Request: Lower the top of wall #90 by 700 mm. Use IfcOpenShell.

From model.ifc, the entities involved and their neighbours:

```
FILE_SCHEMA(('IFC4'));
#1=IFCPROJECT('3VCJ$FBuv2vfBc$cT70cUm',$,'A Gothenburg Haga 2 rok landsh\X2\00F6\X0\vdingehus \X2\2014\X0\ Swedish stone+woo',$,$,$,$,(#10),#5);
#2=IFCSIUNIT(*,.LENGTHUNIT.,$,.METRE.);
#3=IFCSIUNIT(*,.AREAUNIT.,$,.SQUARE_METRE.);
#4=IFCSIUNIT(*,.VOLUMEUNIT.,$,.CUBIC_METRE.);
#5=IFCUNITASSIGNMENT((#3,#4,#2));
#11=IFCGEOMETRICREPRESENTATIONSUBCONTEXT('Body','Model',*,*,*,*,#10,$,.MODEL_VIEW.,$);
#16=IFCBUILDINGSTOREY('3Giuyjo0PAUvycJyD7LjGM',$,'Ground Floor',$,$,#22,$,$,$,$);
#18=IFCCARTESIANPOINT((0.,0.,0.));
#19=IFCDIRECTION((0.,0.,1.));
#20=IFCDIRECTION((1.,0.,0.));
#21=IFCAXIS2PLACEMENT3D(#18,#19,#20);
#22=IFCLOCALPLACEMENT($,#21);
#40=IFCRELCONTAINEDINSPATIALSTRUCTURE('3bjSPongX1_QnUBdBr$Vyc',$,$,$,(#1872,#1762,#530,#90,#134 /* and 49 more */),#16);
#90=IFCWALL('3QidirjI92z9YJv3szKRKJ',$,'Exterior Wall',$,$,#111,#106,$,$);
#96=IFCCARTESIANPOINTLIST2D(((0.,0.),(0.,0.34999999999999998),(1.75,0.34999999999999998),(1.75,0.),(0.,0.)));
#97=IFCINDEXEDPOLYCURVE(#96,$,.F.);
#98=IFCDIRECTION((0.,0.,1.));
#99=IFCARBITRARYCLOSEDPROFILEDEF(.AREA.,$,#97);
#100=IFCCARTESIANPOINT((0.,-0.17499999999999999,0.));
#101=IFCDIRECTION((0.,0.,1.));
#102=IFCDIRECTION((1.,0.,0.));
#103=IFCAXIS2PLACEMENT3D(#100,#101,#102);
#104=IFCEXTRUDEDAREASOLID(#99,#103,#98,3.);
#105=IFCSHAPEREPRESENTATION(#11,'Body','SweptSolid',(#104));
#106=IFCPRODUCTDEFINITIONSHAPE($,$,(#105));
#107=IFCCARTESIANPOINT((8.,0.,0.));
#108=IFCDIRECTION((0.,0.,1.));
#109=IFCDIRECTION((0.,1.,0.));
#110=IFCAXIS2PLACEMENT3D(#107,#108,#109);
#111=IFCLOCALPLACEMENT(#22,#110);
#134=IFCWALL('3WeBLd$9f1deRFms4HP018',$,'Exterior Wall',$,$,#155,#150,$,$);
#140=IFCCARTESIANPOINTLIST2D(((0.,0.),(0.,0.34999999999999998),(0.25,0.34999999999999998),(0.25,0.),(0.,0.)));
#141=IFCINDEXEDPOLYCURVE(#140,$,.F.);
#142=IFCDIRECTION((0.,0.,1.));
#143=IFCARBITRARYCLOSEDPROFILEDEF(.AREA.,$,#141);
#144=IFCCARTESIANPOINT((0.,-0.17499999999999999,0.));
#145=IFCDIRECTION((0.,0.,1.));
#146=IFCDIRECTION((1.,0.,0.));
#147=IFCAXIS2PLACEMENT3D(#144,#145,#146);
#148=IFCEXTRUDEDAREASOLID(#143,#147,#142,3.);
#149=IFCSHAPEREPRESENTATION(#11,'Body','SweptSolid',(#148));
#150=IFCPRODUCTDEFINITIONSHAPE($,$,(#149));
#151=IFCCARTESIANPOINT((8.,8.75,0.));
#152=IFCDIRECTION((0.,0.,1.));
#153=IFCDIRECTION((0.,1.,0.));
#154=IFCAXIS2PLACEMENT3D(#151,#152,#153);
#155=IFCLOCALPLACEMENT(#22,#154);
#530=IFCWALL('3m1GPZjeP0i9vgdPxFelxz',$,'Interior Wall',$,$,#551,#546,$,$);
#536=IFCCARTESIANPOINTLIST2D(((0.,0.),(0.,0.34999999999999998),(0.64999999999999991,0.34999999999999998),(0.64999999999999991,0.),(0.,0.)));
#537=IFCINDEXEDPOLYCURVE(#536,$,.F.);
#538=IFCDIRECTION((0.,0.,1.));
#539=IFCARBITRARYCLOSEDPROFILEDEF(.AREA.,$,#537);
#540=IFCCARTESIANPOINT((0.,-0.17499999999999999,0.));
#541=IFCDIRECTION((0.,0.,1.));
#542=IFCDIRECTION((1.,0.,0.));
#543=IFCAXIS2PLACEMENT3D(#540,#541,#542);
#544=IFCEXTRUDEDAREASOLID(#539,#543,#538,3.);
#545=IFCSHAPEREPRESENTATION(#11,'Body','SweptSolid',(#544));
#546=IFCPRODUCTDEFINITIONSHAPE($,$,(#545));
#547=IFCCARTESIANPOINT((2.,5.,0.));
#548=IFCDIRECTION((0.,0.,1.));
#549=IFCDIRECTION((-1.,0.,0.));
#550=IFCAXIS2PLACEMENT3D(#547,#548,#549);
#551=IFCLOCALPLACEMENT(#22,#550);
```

```python
import ifcopenshell
import ifcopenshell.geom
import ifcopenshell.util.representation
import ifcopenshell.util.shape
import ifcopenshell.util.unit

model = ifcopenshell.open("model.ifc")
unit_scale = ifcopenshell.util.unit.calculate_unit_scale(model)
settings = ifcopenshell.geom.settings()


def volume(element):
    """Net volume in cubic metres, openings subtracted."""
    shape = ifcopenshell.geom.create_shape(settings, element)
    return ifcopenshell.util.shape.get_volume(shape.geometry)


wall = model.by_id(90)
before = volume(wall)

body = ifcopenshell.util.representation.get_representation(wall, "Model", "Body")
solid = body.Items[0]
old_height = solid.Depth
solid.Depth -= 0.7 / unit_scale
after = volume(wall)

print(f"height {old_height:g} -> {solid.Depth:g}, volume {before:.3f} -> {after:.3f} m3")

model.write("model_edited.ifc")
```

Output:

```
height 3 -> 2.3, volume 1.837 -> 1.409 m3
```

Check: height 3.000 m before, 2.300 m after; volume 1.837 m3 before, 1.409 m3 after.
